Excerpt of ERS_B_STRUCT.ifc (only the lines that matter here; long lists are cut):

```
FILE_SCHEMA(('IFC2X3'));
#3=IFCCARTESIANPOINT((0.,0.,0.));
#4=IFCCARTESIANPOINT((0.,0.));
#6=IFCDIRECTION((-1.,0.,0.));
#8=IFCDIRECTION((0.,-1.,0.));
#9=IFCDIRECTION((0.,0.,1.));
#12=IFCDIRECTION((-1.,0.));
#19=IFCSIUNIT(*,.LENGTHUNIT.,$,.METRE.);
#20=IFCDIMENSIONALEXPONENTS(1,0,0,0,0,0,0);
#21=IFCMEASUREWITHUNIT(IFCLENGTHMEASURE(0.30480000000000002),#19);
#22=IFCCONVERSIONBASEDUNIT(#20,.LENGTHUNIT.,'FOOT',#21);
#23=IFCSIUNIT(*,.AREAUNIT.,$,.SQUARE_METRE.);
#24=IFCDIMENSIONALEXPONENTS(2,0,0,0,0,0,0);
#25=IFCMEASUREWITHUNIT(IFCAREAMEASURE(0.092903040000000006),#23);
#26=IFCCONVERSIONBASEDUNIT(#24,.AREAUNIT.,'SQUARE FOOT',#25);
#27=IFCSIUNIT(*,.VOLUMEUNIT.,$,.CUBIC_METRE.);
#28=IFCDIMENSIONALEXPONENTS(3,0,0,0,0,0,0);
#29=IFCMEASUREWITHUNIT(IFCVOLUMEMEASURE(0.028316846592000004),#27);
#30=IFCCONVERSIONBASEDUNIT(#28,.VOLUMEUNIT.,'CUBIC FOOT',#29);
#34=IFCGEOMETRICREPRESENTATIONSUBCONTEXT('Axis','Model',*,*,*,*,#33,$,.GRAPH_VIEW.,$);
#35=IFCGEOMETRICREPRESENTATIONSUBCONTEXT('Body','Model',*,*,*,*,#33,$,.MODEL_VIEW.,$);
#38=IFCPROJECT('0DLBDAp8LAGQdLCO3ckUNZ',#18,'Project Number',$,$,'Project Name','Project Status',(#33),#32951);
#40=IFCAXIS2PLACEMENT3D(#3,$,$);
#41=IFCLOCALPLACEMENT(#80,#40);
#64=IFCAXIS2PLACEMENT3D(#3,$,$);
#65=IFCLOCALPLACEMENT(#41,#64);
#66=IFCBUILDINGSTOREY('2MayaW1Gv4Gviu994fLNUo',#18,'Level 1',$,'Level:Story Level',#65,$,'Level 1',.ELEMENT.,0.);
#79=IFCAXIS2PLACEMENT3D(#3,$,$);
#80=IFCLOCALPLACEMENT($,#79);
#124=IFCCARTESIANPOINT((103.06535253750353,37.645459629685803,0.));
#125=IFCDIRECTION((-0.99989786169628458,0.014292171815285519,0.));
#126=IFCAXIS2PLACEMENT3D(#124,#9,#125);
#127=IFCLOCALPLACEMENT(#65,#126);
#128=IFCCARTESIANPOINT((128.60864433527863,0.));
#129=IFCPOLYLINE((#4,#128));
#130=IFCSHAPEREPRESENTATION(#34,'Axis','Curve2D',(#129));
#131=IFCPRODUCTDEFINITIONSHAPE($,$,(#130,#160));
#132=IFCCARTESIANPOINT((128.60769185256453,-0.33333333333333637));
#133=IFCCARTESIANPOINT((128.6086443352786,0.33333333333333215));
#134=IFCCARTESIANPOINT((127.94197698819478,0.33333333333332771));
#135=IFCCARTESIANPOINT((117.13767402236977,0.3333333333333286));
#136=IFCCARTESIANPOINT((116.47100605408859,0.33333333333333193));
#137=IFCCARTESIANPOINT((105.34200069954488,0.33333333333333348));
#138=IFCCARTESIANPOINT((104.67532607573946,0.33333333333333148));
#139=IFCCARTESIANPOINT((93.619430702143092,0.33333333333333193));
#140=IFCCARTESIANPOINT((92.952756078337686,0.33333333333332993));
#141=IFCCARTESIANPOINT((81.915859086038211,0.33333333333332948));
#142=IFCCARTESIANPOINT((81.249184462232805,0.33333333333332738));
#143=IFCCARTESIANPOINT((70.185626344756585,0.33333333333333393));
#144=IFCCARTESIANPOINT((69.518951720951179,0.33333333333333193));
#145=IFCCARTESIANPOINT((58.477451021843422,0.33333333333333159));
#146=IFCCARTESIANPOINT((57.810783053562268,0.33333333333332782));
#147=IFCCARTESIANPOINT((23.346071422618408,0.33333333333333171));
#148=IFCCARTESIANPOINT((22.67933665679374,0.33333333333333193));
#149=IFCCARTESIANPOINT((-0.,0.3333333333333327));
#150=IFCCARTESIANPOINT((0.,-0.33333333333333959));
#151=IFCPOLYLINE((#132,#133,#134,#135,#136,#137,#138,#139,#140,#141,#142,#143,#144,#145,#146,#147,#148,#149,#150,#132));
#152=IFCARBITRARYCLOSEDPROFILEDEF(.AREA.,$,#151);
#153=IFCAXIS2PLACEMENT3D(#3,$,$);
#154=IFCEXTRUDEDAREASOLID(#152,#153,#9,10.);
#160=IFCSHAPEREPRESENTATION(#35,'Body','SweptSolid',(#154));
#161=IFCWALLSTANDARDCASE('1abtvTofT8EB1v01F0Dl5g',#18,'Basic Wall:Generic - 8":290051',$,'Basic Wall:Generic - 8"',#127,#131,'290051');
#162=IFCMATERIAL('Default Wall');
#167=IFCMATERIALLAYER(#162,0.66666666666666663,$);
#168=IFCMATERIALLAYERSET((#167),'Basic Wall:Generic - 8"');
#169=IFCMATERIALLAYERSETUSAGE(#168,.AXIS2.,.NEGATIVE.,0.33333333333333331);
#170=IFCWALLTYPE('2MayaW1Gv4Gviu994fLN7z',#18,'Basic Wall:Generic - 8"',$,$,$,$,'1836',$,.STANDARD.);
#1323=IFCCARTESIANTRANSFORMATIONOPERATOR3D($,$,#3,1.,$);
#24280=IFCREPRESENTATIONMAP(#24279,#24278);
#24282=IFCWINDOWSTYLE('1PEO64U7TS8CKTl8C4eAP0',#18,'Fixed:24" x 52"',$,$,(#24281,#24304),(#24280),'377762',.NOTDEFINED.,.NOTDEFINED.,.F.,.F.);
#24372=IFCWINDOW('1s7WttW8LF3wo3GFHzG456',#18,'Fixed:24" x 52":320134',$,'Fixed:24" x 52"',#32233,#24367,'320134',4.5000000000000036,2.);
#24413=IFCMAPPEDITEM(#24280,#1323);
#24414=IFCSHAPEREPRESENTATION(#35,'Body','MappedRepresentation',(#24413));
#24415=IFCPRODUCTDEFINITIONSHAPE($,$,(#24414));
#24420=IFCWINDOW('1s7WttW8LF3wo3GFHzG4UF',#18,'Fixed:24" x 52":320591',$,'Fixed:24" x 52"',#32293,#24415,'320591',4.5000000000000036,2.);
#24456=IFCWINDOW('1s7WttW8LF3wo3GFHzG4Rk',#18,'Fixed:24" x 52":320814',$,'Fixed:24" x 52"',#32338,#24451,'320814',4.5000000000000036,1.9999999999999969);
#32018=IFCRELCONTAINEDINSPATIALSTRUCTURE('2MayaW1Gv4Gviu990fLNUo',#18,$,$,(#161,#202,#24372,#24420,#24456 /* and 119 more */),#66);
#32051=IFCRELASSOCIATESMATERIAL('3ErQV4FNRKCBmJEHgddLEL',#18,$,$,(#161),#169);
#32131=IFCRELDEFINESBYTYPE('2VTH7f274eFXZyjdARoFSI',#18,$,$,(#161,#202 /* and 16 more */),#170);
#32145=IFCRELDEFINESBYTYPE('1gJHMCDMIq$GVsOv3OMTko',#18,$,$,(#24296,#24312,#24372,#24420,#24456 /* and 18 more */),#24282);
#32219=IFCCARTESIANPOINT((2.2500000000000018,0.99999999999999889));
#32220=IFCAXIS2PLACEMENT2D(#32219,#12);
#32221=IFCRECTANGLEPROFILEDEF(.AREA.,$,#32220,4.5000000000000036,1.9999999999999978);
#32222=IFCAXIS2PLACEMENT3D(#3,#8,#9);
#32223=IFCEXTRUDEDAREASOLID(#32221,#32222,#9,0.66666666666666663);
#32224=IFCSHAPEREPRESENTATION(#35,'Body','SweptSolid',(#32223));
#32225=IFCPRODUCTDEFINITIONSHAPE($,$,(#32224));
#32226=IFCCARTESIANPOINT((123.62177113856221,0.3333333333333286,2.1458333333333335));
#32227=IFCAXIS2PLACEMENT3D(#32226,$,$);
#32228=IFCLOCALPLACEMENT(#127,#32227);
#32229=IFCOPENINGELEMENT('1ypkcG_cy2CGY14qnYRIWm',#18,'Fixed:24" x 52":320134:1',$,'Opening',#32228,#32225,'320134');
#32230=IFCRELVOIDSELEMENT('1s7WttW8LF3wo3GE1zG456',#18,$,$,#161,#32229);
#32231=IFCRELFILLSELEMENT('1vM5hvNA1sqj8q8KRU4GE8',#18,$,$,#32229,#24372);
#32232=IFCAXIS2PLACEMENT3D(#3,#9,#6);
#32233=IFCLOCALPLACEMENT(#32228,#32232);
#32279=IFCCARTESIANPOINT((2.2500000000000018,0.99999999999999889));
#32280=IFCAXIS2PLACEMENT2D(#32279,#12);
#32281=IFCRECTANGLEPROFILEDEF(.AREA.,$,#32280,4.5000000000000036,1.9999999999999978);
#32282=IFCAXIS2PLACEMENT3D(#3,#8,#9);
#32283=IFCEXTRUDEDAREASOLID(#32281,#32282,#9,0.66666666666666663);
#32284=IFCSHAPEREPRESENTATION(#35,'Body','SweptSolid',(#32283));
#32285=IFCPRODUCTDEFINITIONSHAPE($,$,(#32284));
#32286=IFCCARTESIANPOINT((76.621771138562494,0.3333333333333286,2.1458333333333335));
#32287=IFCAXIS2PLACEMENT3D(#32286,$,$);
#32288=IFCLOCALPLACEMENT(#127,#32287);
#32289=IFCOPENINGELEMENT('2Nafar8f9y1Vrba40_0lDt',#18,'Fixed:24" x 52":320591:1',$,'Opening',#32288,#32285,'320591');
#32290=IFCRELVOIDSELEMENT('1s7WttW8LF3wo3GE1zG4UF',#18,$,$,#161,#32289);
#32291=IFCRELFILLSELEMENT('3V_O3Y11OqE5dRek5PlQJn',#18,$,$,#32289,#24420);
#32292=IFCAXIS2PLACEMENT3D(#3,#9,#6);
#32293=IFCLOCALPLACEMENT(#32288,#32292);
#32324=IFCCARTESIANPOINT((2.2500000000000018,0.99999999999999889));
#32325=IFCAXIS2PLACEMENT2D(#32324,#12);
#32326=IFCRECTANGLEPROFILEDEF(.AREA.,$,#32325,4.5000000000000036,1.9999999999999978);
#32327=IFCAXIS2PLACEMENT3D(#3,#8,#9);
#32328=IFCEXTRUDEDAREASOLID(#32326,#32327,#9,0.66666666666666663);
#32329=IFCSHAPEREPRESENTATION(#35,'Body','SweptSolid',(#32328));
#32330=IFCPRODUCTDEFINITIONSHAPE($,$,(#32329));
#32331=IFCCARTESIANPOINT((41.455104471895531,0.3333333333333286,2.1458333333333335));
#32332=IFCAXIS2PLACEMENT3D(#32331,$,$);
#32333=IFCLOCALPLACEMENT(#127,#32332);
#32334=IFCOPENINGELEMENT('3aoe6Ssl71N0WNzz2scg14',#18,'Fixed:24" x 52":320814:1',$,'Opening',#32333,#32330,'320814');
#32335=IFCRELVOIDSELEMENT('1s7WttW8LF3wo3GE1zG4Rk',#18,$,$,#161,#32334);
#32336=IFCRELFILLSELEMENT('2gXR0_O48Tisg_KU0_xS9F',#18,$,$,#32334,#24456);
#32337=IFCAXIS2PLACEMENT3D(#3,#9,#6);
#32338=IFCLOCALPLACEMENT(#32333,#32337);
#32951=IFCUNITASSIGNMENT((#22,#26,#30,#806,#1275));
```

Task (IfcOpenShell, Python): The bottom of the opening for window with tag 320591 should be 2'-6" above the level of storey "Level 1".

```python
import numpy as np
import ifcopenshell
import ifcopenshell.api.geometry
import ifcopenshell.geom
import ifcopenshell.util.element
import ifcopenshell.util.placement
import ifcopenshell.util.shape
import ifcopenshell.util.unit

model = ifcopenshell.open("ERS_B_STRUCT.ifc")
unit_scale = ifcopenshell.util.unit.calculate_unit_scale(model)

window = model.by_id(24420)
opening = window.FillsVoids[0].RelatingOpeningElement
storey = ifcopenshell.util.element.get_container(window, ifc_class="IfcBuildingStorey")
level = ifcopenshell.util.placement.get_local_placement(storey.ObjectPlacement)[2, 3]

# The opening's origin need not be at the sill, so measure its lowest point.
shape = ifcopenshell.geom.create_shape(ifcopenshell.geom.settings(), opening)
bottom = ifcopenshell.util.shape.get_shape_bottom_elevation(shape, shape.geometry) / unit_scale
dz = level + 30 * 0.0254 / unit_scale - bottom

shift = np.array([0.0, 0.0, dz])
# The window is placed relative to its opening, so it follows when the opening moves.
matrix = ifcopenshell.util.placement.get_local_placement(opening.ObjectPlacement)
matrix[:3, 3] += shift
ifcopenshell.api.geometry.edit_object_placement(
    model, product=opening, matrix=matrix, is_si=False, should_transform_children=True
)

print(f"moved by {dz * unit_scale:+.3f} m")

model.write("ERS_B_STRUCT-out.ifc")
```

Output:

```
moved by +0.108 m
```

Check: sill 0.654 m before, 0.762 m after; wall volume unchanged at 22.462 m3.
